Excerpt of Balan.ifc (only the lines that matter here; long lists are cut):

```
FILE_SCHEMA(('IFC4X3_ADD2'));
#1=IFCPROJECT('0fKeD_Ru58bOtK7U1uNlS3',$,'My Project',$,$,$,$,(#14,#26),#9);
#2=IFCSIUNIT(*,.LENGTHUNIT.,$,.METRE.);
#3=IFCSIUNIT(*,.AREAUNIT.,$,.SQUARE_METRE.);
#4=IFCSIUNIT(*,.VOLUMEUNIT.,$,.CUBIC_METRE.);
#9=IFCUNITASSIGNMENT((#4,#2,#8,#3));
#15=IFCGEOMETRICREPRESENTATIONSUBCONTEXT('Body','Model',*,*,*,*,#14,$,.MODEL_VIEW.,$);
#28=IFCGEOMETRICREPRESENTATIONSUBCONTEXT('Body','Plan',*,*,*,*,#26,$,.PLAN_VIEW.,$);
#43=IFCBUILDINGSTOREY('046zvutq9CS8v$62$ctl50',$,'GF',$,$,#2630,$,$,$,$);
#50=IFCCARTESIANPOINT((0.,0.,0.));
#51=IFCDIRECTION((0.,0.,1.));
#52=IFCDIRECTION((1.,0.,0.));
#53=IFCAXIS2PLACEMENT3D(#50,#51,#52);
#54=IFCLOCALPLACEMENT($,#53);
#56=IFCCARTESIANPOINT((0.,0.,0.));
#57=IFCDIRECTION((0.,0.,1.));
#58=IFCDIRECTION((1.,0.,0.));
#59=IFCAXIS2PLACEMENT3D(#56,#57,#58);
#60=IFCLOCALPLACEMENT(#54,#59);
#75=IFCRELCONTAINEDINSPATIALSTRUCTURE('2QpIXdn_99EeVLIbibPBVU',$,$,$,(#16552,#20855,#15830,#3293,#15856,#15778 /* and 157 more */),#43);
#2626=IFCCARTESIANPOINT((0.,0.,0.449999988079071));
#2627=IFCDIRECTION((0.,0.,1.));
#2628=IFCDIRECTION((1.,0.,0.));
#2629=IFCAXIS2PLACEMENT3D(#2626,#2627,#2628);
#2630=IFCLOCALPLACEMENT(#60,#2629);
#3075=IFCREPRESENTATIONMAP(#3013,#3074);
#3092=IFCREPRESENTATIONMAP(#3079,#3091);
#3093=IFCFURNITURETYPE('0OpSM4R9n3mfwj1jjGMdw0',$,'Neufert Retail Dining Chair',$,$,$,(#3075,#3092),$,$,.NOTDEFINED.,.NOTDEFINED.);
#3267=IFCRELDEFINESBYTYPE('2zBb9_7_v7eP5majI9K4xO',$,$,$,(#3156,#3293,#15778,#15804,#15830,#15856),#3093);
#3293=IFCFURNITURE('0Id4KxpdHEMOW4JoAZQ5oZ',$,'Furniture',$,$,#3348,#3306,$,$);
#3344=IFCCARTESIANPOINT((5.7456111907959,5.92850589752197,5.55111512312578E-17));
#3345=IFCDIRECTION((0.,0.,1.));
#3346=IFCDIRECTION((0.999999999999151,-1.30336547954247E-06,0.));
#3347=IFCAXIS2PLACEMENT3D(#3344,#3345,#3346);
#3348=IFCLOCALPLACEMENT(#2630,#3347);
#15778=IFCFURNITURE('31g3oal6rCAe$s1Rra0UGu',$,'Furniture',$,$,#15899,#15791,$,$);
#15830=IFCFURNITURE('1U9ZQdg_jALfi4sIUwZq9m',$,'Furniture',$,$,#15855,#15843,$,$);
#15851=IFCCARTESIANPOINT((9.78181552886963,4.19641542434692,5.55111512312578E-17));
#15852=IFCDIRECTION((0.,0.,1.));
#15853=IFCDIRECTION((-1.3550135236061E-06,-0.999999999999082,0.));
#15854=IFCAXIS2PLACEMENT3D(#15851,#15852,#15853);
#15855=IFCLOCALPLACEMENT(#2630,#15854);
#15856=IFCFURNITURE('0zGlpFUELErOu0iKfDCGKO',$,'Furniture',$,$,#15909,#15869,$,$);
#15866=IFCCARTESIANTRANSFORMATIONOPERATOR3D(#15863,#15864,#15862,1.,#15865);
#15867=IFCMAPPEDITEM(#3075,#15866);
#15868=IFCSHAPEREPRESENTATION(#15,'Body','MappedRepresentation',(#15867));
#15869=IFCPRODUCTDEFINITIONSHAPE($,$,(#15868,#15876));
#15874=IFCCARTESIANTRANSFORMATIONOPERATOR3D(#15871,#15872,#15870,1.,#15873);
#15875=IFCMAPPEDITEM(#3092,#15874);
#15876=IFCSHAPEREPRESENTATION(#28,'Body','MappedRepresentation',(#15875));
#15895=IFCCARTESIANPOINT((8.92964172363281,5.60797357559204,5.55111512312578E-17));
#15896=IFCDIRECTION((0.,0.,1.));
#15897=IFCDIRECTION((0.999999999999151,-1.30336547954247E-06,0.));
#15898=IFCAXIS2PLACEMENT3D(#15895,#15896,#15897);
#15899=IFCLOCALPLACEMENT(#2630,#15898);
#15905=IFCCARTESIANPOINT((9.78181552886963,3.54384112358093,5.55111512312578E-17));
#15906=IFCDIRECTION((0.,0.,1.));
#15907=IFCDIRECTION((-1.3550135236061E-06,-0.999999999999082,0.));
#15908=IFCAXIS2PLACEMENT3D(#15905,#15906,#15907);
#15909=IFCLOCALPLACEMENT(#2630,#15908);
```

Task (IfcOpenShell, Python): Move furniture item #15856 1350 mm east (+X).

```python
import ifcopenshell
import ifcopenshell.api.geometry
import ifcopenshell.util.placement

model = ifcopenshell.open("Balan.ifc")

item = model.by_guid("0zGlpFUELErOu0iKfDCGKO")
matrix = ifcopenshell.util.placement.get_local_placement(item.ObjectPlacement)
matrix[0, 3] += 1.35
ifcopenshell.api.geometry.edit_object_placement(model, product=item, matrix=matrix, is_si=False)

print(ifcopenshell.util.placement.get_local_placement(item.ObjectPlacement).round(3) + 0.0)

model.write("Balan_edited.ifc")
```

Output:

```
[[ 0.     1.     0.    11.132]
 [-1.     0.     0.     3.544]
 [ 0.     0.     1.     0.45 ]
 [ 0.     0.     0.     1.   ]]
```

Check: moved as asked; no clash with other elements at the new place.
